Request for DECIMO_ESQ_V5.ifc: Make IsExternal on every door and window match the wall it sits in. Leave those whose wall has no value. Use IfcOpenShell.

First a look at what the model holds.

```python
import ifcopenshell
import ifcopenshell.util.element

model = ifcopenshell.open("DECIMO_ESQ_V5.ifc")
print(model.schema)
seen = {}
for e in model.by_type("IfcDoor") + model.by_type("IfcWindow"):
    if not e.FillsVoids:
        continue
    host = e.FillsVoids[0].RelatingOpeningElement.VoidsElements[0].RelatingBuildingElement
    own = ifcopenshell.util.element.get_pset(e, f"Pset_{e.is_a()[3:].removesuffix('StandardCase')}Common", "IsExternal")
    wall = ifcopenshell.util.element.get_pset(host, "Pset_WallCommon", "IsExternal")
    seen[e.is_a(), own, wall] = seen.get((e.is_a(), own, wall), 0) + 1
for (cls, own, wall), count in sorted(seen.items(), key=str):
    print(count, cls, "IsExternal:", own, "| host wall:", wall)
```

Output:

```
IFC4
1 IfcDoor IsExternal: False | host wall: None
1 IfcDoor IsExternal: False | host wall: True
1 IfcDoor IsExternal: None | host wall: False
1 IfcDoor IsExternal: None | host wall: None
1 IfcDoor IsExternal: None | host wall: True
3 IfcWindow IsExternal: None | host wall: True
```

```python
import ifcopenshell
import ifcopenshell.api.pset
import ifcopenshell.util.element

model = ifcopenshell.open("DECIMO_ESQ_V5.ifc")

count = 0
for ifc_class, pset_name in (("IfcDoor", "Pset_DoorCommon"), ("IfcWindow", "Pset_WindowCommon")):
    for e in model.by_type(ifc_class):
        if not e.FillsVoids:
            continue
        host = e.FillsVoids[0].RelatingOpeningElement.VoidsElements[0].RelatingBuildingElement
        external = ifcopenshell.util.element.get_pset(host, "Pset_WallCommon", "IsExternal")
        if external is None or ifcopenshell.util.element.get_pset(e, pset_name, "IsExternal") == external:
            continue
        pset = ifcopenshell.api.pset.add_pset(model, product=e, name=pset_name)
        ifcopenshell.api.pset.edit_pset(model, pset=pset, properties={"IsExternal": external})
        count += 1

print(count, "updated")

model.write("DECIMO_ESQ_V5-out.ifc")
```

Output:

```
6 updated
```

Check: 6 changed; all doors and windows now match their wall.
